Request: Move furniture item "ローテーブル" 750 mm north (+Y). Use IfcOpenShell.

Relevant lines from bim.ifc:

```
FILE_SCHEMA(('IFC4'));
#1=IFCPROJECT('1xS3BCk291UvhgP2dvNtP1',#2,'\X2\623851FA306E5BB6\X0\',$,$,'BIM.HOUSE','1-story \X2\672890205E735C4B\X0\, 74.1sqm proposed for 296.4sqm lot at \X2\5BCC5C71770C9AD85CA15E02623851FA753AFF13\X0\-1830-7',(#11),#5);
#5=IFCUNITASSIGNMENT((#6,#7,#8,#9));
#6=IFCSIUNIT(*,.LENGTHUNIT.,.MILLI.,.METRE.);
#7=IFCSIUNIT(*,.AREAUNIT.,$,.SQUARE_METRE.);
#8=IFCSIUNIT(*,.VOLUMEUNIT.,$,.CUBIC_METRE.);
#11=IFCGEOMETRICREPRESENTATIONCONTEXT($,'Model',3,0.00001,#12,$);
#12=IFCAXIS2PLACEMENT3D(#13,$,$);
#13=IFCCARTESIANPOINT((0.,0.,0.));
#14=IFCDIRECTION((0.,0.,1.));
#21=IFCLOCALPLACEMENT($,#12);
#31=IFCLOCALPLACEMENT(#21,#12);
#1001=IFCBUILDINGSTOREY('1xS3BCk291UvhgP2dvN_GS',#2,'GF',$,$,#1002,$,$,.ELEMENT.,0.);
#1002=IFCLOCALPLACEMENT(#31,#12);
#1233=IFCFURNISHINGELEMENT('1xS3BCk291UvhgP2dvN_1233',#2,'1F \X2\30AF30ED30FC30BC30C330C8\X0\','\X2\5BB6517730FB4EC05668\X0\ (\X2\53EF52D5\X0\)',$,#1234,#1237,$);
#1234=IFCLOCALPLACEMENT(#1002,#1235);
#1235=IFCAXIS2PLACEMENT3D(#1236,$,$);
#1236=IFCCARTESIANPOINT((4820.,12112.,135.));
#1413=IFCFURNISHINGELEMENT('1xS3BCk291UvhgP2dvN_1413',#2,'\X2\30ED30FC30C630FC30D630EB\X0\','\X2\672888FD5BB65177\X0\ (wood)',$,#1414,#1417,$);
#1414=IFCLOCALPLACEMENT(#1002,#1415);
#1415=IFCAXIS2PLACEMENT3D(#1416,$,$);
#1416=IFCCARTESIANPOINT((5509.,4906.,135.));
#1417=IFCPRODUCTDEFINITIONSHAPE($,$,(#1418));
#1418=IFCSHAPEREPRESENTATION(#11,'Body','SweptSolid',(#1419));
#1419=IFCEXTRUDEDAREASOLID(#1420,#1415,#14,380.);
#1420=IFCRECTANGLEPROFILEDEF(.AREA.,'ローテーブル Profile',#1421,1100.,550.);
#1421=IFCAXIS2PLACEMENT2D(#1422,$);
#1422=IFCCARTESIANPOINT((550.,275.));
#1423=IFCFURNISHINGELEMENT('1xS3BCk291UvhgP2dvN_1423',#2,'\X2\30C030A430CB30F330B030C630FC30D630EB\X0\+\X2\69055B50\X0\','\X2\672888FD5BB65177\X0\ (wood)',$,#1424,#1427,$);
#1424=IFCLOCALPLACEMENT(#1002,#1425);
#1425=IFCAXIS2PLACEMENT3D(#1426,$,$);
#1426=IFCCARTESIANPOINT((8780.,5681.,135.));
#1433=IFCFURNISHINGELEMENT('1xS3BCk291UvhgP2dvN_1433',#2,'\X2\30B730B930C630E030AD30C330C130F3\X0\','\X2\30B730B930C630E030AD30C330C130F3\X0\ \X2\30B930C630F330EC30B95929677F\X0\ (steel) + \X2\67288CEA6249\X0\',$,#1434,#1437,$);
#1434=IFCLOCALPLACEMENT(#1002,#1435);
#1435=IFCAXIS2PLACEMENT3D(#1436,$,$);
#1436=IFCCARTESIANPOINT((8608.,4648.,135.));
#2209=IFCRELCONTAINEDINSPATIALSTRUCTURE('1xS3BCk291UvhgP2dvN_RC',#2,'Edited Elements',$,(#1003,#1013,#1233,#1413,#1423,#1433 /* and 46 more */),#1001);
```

```python
import ifcopenshell
import ifcopenshell.api.geometry
import ifcopenshell.util.placement
import ifcopenshell.util.unit

model = ifcopenshell.open("bim.ifc")
unit_scale = ifcopenshell.util.unit.calculate_unit_scale(model)

item = model.by_id(1413)
matrix = ifcopenshell.util.placement.get_local_placement(item.ObjectPlacement)
matrix[1, 3] += 0.75 / unit_scale
ifcopenshell.api.geometry.edit_object_placement(model, product=item, matrix=matrix, is_si=False)

print(ifcopenshell.util.placement.get_local_placement(item.ObjectPlacement).round(3) + 0.0)

model.write("bim_rev.ifc")
```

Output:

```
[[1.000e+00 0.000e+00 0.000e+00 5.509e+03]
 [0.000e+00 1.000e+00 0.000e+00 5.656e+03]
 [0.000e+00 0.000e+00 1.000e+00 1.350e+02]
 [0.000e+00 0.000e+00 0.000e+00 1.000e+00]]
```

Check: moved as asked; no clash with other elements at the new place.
